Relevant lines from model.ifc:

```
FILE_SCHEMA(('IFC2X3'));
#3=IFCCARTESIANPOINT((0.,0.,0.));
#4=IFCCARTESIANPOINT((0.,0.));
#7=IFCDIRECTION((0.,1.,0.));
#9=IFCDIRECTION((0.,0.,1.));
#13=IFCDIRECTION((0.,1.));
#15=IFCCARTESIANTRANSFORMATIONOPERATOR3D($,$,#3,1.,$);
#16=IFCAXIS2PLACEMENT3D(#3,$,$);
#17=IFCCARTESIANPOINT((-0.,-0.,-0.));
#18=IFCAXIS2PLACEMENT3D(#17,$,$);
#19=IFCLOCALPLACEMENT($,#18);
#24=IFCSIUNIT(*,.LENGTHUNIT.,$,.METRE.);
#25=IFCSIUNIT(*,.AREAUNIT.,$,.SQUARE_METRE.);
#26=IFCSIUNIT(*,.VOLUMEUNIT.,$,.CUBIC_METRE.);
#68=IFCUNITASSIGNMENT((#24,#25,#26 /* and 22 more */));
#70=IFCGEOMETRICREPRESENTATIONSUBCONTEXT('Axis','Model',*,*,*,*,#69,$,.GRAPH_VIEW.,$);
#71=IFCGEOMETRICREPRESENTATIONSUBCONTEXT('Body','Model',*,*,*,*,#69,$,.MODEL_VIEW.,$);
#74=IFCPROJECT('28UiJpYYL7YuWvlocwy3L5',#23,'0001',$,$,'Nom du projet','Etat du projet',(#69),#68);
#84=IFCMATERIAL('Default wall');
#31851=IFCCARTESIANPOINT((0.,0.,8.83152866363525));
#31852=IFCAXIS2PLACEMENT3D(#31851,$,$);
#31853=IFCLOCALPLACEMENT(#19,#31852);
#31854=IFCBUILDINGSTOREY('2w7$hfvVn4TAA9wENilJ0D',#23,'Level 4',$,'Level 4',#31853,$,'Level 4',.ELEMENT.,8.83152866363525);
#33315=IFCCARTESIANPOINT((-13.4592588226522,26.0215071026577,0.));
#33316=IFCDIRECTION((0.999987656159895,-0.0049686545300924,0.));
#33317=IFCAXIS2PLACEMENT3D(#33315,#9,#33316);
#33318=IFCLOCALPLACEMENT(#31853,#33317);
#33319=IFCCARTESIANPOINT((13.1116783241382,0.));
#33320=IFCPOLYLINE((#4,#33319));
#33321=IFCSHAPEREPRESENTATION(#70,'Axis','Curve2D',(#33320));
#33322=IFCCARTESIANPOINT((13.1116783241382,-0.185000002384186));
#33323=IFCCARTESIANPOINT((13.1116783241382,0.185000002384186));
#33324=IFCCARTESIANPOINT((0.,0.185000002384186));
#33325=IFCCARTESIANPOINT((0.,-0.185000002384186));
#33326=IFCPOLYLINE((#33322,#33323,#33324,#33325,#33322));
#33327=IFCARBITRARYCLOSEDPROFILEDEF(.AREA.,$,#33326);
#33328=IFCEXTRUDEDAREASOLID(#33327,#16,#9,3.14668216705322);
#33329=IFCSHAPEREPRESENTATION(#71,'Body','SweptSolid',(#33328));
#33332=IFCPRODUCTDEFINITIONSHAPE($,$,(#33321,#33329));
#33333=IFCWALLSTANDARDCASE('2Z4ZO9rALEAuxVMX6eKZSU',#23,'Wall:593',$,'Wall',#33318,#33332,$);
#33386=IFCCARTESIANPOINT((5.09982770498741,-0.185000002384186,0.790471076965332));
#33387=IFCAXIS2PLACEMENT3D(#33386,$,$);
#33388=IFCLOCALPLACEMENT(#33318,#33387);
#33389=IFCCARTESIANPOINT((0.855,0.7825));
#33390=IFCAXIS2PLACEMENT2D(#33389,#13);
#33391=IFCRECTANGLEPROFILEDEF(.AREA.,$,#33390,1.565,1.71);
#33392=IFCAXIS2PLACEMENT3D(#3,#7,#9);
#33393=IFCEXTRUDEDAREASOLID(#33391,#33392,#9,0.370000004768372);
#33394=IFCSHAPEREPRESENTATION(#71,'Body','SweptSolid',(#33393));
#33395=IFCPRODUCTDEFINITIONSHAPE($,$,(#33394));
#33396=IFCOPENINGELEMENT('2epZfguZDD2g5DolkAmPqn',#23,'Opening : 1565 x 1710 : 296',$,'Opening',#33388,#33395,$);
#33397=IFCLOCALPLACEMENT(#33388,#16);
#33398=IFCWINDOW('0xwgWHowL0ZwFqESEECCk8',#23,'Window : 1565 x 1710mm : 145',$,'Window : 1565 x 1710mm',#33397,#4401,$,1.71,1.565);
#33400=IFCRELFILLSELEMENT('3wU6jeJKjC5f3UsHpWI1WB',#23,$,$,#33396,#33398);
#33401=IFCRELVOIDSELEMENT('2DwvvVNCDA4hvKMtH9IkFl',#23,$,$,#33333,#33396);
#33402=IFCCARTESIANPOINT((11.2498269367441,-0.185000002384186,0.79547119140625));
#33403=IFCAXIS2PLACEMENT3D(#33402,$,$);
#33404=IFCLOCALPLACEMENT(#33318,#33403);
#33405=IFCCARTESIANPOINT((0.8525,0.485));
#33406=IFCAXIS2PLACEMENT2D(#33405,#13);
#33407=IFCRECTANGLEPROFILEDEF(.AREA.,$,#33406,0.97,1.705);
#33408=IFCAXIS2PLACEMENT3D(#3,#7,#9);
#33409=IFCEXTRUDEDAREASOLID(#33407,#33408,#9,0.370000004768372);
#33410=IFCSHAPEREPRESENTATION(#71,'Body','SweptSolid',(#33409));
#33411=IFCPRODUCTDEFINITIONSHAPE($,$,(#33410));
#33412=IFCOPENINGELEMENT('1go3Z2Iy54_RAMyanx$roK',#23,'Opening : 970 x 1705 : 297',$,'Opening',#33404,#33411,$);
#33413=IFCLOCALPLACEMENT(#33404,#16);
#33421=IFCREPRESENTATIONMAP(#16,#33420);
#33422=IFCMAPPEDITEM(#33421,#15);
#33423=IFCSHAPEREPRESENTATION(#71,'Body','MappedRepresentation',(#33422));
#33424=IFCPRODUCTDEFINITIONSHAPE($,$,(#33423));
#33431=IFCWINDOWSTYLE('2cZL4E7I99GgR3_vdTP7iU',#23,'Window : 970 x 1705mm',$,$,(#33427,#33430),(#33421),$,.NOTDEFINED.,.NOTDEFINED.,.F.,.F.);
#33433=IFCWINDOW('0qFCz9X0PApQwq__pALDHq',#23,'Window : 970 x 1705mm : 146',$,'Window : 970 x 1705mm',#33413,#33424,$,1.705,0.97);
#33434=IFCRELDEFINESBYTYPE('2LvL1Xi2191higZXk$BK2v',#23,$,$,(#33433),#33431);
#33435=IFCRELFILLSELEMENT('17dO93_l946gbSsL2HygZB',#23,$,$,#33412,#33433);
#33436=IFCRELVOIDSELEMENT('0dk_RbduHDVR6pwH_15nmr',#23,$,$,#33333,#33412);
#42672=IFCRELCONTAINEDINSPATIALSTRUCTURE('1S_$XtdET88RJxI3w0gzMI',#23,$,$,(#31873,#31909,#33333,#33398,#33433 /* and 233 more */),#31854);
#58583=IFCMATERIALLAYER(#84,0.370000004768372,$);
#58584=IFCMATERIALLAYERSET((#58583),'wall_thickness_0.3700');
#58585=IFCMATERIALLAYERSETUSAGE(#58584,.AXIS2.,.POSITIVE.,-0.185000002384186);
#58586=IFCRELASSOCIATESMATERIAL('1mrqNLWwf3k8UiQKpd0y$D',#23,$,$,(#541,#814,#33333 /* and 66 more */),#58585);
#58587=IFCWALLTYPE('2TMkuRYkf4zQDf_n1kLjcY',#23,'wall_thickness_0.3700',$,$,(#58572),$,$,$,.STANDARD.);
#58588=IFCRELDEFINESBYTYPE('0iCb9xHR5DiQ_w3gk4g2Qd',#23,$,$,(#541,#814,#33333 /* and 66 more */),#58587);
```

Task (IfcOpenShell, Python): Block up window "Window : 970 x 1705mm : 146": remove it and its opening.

```python
import ifcopenshell
import ifcopenshell.api.feature
import ifcopenshell.api.root
import ifcopenshell.geom
import ifcopenshell.util.shape

model = ifcopenshell.open("model.ifc")
settings = ifcopenshell.geom.settings()


def volume(element):
    """Net volume in cubic metres, openings subtracted."""
    shape = ifcopenshell.geom.create_shape(settings, element)
    return ifcopenshell.util.shape.get_volume(shape.geometry)


window = model.by_guid("0qFCz9X0PApQwq__pALDHq")
opening = window.FillsVoids[0].RelatingOpeningElement
wall = opening.VoidsElements[0].RelatingBuildingElement
before = volume(wall)

ifcopenshell.api.root.remove_product(model, product=window)
ifcopenshell.api.feature.remove_feature(model, feature=opening)

after = volume(wall)

print(f"wall volume {before:.3f} -> {after:.3f} m3")

model.write("model_v2.ifc")
```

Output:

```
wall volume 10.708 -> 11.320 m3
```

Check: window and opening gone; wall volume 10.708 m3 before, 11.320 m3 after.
